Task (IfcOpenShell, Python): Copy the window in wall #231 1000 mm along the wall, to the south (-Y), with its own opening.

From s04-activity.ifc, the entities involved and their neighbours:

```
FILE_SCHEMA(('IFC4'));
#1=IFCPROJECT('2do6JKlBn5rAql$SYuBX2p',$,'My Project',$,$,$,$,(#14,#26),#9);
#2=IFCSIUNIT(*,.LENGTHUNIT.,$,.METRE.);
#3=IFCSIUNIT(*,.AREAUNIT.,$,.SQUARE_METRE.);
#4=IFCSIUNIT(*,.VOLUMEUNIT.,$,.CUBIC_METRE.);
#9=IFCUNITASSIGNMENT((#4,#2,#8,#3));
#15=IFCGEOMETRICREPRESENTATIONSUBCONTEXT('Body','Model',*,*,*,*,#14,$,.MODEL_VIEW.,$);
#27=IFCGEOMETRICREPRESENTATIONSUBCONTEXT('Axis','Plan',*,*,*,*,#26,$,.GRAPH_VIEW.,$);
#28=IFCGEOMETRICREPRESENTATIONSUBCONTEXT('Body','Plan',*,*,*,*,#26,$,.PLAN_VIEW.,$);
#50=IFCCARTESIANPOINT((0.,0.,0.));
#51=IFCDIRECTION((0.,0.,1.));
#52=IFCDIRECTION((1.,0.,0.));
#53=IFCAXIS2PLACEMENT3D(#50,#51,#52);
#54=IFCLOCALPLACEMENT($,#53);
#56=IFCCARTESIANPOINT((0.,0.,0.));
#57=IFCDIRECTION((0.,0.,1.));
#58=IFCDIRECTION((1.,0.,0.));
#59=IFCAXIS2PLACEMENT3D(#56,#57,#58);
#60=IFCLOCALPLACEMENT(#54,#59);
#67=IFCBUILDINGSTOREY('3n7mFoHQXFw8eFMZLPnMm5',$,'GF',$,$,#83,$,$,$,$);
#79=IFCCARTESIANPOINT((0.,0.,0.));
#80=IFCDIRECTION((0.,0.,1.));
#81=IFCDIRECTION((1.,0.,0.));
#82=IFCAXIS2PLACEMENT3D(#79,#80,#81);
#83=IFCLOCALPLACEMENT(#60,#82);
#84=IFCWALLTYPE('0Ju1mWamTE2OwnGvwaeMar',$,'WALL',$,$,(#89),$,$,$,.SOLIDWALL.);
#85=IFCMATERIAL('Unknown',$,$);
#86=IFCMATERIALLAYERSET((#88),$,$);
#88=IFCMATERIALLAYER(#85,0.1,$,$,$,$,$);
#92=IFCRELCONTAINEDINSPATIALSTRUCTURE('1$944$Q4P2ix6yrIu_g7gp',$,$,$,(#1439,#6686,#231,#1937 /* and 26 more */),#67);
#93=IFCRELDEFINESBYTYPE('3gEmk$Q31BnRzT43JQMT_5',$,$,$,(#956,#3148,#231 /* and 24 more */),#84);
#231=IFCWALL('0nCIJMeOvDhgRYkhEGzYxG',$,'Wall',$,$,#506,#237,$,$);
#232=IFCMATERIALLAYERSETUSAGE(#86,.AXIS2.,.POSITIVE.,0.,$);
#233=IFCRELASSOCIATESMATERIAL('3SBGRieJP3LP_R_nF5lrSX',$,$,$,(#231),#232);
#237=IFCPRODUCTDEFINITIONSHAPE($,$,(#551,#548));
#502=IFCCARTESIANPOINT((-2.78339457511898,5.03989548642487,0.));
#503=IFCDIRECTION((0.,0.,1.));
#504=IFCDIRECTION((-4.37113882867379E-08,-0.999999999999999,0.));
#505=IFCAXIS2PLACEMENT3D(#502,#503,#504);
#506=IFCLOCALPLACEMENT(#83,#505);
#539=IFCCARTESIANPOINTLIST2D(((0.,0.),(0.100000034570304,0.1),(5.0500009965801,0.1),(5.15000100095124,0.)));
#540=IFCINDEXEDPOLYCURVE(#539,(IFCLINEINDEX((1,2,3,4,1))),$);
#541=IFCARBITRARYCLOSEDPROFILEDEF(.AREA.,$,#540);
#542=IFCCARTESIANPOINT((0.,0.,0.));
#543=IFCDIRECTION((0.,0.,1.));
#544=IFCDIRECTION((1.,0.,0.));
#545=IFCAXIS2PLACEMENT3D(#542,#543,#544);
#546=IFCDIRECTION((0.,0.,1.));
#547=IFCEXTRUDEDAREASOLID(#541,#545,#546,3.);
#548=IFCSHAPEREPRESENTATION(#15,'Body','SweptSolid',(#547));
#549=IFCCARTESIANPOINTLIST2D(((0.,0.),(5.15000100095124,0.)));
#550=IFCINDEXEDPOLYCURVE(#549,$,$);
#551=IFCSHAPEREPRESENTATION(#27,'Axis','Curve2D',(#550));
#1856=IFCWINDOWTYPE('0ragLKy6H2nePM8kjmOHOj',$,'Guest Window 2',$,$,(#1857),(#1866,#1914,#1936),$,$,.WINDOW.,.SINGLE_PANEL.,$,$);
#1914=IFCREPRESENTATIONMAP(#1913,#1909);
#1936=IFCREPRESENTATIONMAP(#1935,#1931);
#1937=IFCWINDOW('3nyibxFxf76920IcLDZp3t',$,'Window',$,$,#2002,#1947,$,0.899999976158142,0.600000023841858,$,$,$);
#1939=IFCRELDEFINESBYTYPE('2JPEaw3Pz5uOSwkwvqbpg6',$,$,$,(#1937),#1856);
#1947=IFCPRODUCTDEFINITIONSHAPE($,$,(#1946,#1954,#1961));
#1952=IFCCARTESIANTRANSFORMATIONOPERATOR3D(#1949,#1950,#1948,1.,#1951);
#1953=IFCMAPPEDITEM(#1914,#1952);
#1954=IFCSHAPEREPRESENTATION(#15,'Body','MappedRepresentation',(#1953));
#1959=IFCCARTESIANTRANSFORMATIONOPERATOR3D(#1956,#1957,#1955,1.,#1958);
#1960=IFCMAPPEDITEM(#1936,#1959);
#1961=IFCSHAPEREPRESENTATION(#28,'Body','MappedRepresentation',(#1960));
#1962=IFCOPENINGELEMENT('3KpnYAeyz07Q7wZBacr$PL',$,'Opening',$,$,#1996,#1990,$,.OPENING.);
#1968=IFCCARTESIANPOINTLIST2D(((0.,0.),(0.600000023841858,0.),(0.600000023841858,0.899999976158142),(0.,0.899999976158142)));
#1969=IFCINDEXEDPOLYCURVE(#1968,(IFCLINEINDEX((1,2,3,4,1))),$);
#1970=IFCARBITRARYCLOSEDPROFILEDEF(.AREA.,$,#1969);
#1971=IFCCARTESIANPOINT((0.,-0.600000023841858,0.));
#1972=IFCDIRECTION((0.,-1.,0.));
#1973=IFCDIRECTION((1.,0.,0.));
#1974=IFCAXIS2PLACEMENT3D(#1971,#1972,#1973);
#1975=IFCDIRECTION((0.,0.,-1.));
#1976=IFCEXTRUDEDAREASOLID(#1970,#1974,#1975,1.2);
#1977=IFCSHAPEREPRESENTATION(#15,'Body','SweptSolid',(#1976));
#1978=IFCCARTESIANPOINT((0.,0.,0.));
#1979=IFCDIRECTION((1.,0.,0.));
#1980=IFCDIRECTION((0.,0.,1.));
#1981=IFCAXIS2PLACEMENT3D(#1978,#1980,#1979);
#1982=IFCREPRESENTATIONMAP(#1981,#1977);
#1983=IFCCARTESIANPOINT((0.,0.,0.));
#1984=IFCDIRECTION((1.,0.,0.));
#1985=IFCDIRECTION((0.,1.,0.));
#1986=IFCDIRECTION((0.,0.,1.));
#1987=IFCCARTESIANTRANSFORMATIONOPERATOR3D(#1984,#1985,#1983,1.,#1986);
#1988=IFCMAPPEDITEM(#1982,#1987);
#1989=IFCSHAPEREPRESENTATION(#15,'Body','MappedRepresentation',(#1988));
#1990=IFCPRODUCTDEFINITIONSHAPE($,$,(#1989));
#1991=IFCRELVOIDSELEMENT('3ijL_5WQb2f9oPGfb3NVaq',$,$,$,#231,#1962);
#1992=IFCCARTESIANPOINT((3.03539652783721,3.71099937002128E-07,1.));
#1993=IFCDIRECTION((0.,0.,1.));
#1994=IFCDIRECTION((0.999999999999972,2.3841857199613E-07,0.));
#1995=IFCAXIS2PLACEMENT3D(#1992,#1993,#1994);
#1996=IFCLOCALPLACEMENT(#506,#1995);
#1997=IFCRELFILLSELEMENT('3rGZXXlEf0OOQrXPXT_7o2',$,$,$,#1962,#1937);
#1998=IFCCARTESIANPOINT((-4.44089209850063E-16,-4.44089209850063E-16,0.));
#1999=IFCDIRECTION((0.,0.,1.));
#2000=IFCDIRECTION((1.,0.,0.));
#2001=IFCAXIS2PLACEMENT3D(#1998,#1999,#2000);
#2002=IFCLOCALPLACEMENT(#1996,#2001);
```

```python
import ifcopenshell
import ifcopenshell.api.feature
import ifcopenshell.api.geometry
import ifcopenshell.api.root
import ifcopenshell.geom
import ifcopenshell.util.element
import ifcopenshell.util.placement
import ifcopenshell.util.shape

model = ifcopenshell.open("s04-activity.ifc")
settings = ifcopenshell.geom.settings()


def volume(element):
    """Net volume in cubic metres, openings subtracted."""
    shape = ifcopenshell.geom.create_shape(settings, element)
    return ifcopenshell.util.shape.get_volume(shape.geometry)


window = model.by_guid("3nyibxFxf76920IcLDZp3t")
opening = window.FillsVoids[0].RelatingOpeningElement
wall = opening.VoidsElements[0].RelatingBuildingElement
before = volume(wall)
shift = ifcopenshell.util.placement.get_local_placement(wall.ObjectPlacement)[:3, 0] * 1.0

# copy_class copies the void relationship, type, container and properties, but no geometry.
new_opening = ifcopenshell.api.root.copy_class(model, product=opening)
new_opening.Representation = ifcopenshell.util.element.copy_deep(
    model, opening.Representation, exclude=["IfcGeometricRepresentationContext", "IfcRepresentationMap"]
)
new_window = ifcopenshell.api.root.copy_class(model, product=window)
new_window.Representation = ifcopenshell.util.element.copy_deep(
    model, window.Representation, exclude=["IfcGeometricRepresentationContext", "IfcRepresentationMap"]
)
ifcopenshell.api.feature.add_filling(model, opening=new_opening, element=new_window)

for old, new in ((opening, new_opening), (window, new_window)):
    matrix = ifcopenshell.util.placement.get_local_placement(old.ObjectPlacement)
    matrix[:3, 3] += shift
    ifcopenshell.api.geometry.edit_object_placement(model, product=new, matrix=matrix, is_si=False)

after = volume(wall)

print(f"wall volume {before:.3f} -> {after:.3f} m3")

model.write("s04-activity_v2.ifc")
```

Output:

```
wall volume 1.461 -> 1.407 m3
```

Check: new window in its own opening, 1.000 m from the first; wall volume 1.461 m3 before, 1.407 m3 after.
